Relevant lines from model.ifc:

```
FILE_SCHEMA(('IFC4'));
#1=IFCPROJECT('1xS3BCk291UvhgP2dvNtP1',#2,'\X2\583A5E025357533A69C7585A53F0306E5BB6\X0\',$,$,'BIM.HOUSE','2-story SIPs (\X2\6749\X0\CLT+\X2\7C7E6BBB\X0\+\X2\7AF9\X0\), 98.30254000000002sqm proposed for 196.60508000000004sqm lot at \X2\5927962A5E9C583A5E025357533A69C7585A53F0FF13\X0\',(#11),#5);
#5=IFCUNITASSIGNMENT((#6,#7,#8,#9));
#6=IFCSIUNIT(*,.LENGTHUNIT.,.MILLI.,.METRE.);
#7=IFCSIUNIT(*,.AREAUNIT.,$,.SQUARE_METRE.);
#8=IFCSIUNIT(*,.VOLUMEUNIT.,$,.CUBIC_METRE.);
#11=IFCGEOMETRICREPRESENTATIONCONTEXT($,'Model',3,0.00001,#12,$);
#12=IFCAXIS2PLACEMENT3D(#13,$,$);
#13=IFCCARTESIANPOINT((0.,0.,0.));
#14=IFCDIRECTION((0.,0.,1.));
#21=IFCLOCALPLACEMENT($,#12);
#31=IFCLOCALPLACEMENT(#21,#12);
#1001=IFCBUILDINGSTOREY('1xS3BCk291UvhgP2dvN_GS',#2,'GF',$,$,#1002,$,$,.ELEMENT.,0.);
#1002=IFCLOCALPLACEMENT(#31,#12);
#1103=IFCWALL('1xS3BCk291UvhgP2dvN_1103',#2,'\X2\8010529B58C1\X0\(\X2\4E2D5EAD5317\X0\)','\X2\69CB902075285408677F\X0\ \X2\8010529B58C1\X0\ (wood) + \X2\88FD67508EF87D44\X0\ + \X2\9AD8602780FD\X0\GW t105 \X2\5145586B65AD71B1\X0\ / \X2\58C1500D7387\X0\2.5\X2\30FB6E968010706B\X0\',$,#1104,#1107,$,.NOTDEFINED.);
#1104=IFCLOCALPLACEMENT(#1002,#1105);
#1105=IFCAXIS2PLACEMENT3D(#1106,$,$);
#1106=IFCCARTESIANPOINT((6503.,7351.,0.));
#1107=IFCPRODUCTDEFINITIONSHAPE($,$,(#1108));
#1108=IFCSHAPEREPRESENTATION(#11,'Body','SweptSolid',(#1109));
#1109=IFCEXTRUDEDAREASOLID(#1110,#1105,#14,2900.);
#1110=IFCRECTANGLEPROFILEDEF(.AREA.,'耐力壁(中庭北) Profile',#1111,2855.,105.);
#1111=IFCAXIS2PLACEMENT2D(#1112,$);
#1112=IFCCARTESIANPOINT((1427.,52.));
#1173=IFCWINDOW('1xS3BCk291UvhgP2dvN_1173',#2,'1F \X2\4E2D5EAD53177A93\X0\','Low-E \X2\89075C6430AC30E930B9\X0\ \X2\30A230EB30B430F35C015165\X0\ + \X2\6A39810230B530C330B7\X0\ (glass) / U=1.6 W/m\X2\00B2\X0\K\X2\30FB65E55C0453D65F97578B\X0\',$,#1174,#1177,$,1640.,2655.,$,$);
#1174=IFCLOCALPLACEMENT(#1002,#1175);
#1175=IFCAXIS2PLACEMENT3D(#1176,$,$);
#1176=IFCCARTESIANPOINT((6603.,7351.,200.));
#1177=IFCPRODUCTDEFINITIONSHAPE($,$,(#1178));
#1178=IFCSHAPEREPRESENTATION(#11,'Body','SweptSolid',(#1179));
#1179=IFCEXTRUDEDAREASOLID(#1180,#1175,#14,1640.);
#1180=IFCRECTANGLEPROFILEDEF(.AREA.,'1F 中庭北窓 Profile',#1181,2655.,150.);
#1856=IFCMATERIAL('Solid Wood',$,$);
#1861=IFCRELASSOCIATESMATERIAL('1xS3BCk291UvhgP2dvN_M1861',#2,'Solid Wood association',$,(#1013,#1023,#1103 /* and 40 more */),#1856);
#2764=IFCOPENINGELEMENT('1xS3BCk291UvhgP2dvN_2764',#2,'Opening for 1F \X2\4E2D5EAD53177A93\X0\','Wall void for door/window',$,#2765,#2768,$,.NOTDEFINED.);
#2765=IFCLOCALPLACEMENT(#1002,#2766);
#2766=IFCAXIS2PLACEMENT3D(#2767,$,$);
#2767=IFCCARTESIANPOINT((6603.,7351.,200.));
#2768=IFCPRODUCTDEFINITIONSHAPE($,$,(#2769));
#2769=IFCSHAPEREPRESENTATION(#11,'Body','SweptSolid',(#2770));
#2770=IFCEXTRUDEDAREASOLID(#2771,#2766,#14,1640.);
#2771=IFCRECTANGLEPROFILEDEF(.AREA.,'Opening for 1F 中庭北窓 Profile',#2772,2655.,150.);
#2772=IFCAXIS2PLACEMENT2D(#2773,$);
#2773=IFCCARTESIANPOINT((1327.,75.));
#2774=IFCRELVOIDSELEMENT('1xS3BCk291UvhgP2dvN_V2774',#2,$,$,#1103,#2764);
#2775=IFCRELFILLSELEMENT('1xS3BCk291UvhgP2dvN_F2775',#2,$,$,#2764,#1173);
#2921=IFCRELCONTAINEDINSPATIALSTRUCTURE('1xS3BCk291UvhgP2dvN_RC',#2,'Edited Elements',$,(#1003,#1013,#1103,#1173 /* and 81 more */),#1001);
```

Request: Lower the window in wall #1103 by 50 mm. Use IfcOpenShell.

```python
import numpy as np
import ifcopenshell
import ifcopenshell.api.geometry
import ifcopenshell.util.placement
import ifcopenshell.util.unit

model = ifcopenshell.open("model.ifc")
unit_scale = ifcopenshell.util.unit.calculate_unit_scale(model)

window = model.by_guid("1xS3BCk291UvhgP2dvN_1173")
opening = window.FillsVoids[0].RelatingOpeningElement
dz = -50.0

shift = np.array([0.0, 0.0, dz])
# The window is not placed relative to its opening, so move both.
for product in (opening, window):
    matrix = ifcopenshell.util.placement.get_local_placement(product.ObjectPlacement)
    matrix[:3, 3] += shift
    ifcopenshell.api.geometry.edit_object_placement(model, product=product, matrix=matrix, is_si=False)

print(f"moved by {dz * unit_scale:+.3f} m")

model.write("model_rev.ifc")
```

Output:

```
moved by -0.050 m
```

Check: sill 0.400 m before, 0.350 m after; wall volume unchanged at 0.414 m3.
